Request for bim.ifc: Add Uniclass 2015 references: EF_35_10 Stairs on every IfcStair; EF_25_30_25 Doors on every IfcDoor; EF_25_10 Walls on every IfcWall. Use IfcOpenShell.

First a look at what the model holds.

```python
import ifcopenshell

model = ifcopenshell.open("bim.ifc")
print(model.schema)
print("classifications:", [c.Name for c in model.by_type("IfcClassification")])
for ifc_class in ("IfcDoor", "IfcRoof", "IfcStair", "IfcWall", "IfcWindow"):
    print(ifc_class, len(model.by_type(ifc_class)))
```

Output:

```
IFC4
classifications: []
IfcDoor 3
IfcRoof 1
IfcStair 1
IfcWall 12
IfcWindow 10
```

```python
import ifcopenshell
import ifcopenshell.api.classification

model = ifcopenshell.open("bim.ifc")

system = ifcopenshell.api.classification.add_classification(model, classification="Uniclass 2015")

codes = {
    "IfcStair": ("EF_35_10", "Stairs"),
    "IfcDoor": ("EF_25_30_25", "Doors"),
    "IfcWall": ("EF_25_10", "Walls"),
}
for ifc_class, (code, name) in codes.items():
    products = model.by_type(ifc_class)
    ifcopenshell.api.classification.add_reference(
        model, products=products, classification=system, identification=code, name=name
    )
    print(code, len(products))

model.write("bim-out.ifc")
```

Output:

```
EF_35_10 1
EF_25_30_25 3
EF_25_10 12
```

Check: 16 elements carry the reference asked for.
